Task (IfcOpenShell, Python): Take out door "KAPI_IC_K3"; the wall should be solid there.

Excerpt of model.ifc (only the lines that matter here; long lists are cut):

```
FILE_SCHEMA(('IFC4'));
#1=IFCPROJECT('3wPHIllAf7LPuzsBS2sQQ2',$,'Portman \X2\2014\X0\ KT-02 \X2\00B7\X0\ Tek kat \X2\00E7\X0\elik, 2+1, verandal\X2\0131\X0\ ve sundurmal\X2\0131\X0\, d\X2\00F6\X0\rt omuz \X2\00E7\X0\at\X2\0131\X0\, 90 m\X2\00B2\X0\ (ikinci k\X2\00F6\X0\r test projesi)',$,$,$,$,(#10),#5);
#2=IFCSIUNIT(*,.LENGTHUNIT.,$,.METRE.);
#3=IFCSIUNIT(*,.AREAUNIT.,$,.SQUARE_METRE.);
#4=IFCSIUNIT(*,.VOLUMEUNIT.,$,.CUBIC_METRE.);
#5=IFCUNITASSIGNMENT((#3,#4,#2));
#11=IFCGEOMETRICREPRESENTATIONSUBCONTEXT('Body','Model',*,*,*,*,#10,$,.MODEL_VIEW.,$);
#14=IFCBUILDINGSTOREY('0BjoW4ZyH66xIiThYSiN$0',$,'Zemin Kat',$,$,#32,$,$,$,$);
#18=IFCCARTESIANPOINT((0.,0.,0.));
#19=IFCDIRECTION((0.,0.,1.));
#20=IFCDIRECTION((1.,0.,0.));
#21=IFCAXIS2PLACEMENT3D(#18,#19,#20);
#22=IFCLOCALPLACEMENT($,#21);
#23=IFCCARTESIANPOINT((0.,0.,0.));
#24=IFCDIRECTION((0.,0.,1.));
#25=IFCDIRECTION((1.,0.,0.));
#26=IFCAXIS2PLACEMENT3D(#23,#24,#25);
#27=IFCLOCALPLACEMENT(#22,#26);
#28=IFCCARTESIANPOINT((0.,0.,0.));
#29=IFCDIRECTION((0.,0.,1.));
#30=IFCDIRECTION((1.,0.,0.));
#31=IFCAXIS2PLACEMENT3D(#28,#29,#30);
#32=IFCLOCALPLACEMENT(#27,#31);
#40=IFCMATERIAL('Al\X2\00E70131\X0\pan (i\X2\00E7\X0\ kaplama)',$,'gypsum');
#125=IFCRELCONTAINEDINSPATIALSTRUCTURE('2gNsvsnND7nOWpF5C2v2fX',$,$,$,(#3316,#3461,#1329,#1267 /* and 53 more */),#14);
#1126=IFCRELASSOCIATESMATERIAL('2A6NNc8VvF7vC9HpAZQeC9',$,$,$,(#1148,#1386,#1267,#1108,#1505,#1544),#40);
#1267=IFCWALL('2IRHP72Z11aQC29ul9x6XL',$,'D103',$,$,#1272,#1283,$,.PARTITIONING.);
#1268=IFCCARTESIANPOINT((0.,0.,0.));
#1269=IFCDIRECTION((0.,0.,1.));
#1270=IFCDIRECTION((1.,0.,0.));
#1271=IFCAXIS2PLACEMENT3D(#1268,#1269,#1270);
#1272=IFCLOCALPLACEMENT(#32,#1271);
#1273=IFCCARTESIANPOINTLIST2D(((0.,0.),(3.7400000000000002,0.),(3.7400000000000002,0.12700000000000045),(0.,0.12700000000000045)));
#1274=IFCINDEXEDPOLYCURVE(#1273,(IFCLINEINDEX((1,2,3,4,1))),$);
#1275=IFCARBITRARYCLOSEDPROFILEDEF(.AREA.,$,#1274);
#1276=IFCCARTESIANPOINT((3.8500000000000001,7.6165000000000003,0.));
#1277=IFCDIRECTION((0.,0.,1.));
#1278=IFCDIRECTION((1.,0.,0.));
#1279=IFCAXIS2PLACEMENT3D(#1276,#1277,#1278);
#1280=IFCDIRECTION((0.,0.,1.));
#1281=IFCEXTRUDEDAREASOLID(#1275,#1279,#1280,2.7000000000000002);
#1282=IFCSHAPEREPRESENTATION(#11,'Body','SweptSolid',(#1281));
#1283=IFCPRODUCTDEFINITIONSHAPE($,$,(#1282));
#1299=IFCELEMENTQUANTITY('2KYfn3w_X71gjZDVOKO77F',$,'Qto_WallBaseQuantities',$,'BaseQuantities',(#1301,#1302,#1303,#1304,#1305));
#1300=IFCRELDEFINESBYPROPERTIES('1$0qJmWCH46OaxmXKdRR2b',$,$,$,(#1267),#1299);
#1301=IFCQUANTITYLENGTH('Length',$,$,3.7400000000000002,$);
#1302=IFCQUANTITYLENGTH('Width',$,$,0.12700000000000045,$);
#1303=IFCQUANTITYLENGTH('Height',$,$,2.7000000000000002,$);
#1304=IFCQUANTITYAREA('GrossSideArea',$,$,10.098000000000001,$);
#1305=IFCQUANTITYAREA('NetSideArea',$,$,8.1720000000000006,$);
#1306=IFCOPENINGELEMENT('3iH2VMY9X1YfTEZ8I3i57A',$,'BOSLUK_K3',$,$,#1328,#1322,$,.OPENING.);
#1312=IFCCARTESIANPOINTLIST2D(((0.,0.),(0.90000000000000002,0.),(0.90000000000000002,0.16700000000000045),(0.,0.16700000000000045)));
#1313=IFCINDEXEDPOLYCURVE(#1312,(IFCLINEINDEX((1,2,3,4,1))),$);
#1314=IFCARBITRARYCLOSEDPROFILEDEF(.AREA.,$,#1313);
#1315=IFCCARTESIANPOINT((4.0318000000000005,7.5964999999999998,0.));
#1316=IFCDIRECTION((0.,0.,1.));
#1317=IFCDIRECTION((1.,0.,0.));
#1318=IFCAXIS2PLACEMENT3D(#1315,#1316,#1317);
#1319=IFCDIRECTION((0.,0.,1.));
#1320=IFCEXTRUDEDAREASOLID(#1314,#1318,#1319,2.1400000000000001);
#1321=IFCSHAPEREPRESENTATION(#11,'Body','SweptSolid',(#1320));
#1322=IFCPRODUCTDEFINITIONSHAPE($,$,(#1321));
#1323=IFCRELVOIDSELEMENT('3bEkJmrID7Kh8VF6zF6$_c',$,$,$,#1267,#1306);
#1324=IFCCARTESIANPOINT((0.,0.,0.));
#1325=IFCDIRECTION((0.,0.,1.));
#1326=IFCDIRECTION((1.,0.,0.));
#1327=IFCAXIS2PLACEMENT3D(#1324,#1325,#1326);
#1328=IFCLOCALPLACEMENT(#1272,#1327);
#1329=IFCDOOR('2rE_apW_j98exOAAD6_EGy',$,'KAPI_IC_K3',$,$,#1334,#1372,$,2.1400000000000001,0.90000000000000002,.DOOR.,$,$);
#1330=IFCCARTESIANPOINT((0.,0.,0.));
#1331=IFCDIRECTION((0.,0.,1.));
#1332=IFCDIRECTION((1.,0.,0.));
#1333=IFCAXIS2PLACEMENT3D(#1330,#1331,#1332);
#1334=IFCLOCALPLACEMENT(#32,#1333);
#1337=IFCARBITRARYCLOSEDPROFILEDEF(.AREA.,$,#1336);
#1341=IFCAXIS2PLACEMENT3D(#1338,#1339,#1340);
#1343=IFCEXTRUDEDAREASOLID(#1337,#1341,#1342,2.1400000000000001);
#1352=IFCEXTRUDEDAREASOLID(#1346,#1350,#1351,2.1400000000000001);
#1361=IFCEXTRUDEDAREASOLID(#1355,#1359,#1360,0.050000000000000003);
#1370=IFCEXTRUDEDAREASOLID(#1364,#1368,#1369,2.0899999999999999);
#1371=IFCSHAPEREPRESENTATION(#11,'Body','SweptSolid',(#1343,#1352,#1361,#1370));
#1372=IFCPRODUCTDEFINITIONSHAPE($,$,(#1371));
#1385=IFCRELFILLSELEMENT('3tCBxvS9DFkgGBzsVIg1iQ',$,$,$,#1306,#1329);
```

```python
import ifcopenshell
import ifcopenshell.api.feature
import ifcopenshell.api.pset
import ifcopenshell.api.root
import ifcopenshell.geom
import ifcopenshell.util.element
import ifcopenshell.util.shape
import ifcopenshell.util.unit

model = ifcopenshell.open("model.ifc")
area_scale = ifcopenshell.util.unit.calculate_unit_scale(model, "AREAUNIT")
settings = ifcopenshell.geom.settings()


def volume(element):
    """Net volume in cubic metres, openings subtracted."""
    shape = ifcopenshell.geom.create_shape(settings, element)
    return ifcopenshell.util.shape.get_volume(shape.geometry)


door = model.by_guid("2rE_apW_j98exOAAD6_EGy")
opening = door.FillsVoids[0].RelatingOpeningElement
wall = opening.VoidsElements[0].RelatingBuildingElement
before = volume(wall)

ifcopenshell.api.root.remove_product(model, product=door)
ifcopenshell.api.feature.remove_feature(model, feature=opening)

after = volume(wall)
thickness = 0.127  # wall thickness in metres

# Update the wall's stored quantities.
qto = model.by_id(ifcopenshell.util.element.get_pset(wall, "Qto_WallBaseQuantities", should_inherit=False)["id"])
ifcopenshell.api.pset.edit_qto(model, qto=qto, properties={"NetSideArea": after / thickness / area_scale})

print(f"wall volume {before:.3f} -> {after:.3f} m3")

model.write("model_updated.ifc")
```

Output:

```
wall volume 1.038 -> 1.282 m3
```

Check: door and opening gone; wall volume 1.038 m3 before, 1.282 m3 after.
